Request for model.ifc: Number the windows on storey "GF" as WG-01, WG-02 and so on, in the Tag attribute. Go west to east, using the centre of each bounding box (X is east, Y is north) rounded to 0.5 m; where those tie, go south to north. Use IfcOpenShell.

First a look at what the model holds.

```python
import ifcopenshell
import ifcopenshell.util.element
import ifcopenshell.util.placement

model = ifcopenshell.open("model.ifc")
print(model.schema)
storey = next(s for s in model.by_type("IfcBuildingStorey") if s.Name == "GF")
windows = [e for e in ifcopenshell.util.element.get_decomposition(storey) if e.is_a("IfcWindow")]
for e in sorted(windows, key=lambda e: e.id()):
    origin = ifcopenshell.util.placement.get_local_placement(e.ObjectPlacement)[:3, 3]
    print(e.id(), e.Tag, e.Name, origin.round(2) + 0.0, sep=" | ")
```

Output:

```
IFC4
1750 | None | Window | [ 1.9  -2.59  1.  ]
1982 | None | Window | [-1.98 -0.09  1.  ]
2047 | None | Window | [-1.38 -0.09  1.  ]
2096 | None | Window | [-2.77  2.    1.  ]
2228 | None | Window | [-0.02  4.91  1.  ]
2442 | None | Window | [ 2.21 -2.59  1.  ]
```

```python
import ifcopenshell
import ifcopenshell.geom
import ifcopenshell.util.element
import ifcopenshell.util.shape

model = ifcopenshell.open("model.ifc")
settings = ifcopenshell.geom.settings()
settings.set("use-world-coords", True)


def centre(element):
    shape = ifcopenshell.geom.create_shape(settings, element)
    return ifcopenshell.util.shape.get_bbox_centroid(shape.geometry)


storey = next(s for s in model.by_type("IfcBuildingStorey") if s.Name == "GF")
windows = [e for e in ifcopenshell.util.element.get_decomposition(storey) if e.is_a("IfcWindow")]

# Insertion points can sit at a corner or the storey origin, so sort by the geometry (in metres).
centres = {e: centre(e) for e in windows}
windows.sort(key=lambda e: (round(centres[e][0] / 0.5), centres[e][1]))

for i, e in enumerate(windows, start=1):
    number = f"WG-{i:02d}"
    e.Tag = number
    print(e.id(), number)

model.write("model_v2.ifc")
```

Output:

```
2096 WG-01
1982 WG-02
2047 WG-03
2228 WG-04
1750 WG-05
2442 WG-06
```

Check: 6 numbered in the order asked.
